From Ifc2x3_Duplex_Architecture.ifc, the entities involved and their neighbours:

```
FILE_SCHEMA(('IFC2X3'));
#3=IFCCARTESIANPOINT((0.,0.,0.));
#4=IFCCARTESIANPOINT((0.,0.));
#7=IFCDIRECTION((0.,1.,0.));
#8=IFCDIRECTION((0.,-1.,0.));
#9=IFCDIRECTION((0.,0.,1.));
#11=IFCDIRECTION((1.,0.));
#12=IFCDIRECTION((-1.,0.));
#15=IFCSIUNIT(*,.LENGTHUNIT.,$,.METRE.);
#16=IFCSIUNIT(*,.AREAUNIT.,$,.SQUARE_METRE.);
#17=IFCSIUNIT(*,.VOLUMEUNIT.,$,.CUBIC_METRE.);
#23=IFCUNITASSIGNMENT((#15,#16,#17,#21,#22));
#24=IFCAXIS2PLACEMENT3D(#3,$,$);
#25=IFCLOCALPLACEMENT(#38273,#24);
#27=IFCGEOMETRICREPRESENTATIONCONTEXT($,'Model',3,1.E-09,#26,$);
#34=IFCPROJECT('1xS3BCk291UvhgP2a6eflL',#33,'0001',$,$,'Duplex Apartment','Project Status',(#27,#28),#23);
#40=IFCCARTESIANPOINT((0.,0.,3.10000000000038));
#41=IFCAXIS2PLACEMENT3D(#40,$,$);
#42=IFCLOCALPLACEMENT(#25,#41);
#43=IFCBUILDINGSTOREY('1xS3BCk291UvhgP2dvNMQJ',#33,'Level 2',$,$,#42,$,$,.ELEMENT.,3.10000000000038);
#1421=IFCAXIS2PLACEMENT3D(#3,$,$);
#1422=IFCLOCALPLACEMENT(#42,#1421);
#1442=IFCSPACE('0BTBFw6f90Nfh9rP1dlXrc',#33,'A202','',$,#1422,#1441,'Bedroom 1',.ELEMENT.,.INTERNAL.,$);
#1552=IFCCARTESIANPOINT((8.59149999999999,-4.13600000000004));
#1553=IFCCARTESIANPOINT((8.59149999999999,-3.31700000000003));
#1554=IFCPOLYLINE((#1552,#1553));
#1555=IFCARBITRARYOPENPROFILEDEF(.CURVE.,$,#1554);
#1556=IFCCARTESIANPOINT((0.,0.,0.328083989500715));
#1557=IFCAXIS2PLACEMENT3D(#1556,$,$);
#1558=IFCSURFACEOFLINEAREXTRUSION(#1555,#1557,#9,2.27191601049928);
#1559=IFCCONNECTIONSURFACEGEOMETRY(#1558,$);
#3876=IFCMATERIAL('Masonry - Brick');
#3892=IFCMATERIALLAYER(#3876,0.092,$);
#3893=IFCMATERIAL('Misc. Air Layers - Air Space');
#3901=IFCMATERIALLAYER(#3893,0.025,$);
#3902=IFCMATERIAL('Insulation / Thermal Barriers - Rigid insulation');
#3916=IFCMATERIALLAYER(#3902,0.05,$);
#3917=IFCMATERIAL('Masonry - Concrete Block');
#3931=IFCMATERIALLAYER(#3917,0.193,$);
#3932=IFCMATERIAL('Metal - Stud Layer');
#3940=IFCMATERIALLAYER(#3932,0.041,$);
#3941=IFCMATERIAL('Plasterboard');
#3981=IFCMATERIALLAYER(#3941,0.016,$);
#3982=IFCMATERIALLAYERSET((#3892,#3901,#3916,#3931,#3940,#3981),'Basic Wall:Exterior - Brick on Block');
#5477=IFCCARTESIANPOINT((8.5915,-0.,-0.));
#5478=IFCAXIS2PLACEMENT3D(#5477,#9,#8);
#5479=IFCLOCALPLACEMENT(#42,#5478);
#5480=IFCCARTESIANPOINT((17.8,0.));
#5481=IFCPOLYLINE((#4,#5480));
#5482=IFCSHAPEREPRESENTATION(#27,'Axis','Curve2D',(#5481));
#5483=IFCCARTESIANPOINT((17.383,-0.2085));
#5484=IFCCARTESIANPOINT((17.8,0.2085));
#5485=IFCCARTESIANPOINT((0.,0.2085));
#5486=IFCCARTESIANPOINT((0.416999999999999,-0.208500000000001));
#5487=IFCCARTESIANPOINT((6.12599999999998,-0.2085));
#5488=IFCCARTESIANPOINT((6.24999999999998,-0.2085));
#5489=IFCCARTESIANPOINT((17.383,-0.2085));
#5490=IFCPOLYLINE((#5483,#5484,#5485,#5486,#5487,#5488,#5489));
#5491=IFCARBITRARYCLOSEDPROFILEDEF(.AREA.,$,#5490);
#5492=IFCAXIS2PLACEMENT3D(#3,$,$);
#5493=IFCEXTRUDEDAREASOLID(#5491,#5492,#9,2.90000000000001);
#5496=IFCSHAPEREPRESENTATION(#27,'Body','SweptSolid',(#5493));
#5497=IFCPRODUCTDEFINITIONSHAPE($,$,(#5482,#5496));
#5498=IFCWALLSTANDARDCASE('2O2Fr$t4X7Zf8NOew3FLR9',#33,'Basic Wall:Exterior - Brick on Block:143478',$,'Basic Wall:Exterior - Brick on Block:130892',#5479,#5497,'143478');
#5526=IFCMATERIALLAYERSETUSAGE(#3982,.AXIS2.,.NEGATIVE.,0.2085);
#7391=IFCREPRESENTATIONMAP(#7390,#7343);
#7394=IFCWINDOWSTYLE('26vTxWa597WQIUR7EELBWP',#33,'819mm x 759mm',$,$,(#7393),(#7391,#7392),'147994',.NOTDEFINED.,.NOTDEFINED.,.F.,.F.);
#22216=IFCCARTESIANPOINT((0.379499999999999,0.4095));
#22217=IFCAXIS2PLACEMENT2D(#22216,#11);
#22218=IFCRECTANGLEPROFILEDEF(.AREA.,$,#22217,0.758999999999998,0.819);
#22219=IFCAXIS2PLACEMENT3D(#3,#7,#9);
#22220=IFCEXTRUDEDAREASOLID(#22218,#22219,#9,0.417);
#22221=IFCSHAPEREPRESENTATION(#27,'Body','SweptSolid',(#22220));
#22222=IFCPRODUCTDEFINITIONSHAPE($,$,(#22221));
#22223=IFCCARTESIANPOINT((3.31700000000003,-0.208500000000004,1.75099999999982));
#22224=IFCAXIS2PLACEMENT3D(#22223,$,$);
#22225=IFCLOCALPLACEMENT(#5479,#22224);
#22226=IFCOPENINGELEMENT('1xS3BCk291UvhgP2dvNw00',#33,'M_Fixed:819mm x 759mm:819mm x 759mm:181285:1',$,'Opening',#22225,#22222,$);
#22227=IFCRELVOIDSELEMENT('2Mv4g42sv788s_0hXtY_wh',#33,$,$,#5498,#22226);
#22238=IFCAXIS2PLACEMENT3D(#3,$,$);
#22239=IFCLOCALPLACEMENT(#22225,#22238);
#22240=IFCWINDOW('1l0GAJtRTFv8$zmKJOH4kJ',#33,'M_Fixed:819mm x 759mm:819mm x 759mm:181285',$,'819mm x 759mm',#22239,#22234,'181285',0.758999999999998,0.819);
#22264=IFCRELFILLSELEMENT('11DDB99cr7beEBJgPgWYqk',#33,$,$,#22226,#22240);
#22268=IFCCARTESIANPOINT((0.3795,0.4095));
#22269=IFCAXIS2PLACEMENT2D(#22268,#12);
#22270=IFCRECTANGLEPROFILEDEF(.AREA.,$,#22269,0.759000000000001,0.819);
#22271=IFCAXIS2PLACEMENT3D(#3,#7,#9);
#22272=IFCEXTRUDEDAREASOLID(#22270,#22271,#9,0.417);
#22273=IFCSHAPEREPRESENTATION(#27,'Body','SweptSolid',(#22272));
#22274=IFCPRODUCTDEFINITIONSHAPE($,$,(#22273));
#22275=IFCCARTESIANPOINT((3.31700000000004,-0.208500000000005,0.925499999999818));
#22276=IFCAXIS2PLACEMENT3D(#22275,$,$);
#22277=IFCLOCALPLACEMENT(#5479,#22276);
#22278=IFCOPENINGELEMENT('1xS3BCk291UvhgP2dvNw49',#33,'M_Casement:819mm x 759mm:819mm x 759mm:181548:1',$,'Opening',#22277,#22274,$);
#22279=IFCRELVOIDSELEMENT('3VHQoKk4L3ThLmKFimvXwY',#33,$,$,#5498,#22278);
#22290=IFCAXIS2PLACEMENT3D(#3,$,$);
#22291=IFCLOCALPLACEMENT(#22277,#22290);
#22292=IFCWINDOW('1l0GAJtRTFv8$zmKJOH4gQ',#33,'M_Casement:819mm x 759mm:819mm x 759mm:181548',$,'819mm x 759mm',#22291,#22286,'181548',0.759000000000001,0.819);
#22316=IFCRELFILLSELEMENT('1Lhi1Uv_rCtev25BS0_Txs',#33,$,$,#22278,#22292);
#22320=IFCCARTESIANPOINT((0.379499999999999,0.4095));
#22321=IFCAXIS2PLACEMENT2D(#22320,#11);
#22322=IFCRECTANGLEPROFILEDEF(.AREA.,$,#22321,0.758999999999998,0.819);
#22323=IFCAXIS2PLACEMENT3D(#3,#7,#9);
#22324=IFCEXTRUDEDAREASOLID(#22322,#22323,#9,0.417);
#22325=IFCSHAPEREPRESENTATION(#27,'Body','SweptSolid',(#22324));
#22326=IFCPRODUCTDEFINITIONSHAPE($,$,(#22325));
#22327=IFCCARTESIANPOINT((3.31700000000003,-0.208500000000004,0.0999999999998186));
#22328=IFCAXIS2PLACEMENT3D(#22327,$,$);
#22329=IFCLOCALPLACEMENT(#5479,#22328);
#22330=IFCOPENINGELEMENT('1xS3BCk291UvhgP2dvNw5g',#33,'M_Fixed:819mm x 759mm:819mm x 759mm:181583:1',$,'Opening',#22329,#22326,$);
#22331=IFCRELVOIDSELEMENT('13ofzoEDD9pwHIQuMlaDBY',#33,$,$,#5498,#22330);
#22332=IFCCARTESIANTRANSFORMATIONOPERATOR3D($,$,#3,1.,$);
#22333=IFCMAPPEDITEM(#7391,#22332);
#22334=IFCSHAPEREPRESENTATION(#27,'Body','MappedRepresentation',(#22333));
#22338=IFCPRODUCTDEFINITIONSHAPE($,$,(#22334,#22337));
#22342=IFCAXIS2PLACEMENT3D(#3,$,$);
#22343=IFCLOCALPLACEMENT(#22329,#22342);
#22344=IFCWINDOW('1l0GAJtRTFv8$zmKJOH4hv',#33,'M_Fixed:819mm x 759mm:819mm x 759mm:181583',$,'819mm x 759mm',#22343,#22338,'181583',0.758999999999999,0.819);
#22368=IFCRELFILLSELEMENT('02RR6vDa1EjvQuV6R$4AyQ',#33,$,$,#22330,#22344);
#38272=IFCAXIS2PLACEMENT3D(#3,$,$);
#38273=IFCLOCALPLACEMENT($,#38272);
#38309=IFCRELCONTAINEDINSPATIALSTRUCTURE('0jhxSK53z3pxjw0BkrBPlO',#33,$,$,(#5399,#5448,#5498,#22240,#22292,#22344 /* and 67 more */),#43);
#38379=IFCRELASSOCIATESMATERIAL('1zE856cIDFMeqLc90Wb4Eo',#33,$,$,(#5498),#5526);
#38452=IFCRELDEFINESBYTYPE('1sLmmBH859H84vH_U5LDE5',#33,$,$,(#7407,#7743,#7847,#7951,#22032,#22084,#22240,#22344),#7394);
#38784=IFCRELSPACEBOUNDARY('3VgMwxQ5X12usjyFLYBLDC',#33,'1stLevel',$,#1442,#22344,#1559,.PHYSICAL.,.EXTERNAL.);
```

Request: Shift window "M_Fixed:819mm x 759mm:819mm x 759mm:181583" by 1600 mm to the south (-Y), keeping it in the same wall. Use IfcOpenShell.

```python
import numpy as np
import ifcopenshell
import ifcopenshell.api.geometry
import ifcopenshell.util.placement
import ifcopenshell.util.unit

model = ifcopenshell.open("Ifc2x3_Duplex_Architecture.ifc")
unit_scale = ifcopenshell.util.unit.calculate_unit_scale(model)

window = model.by_guid("1l0GAJtRTFv8$zmKJOH4hv")
opening = window.FillsVoids[0].RelatingOpeningElement
wall = opening.VoidsElements[0].RelatingBuildingElement

wall_matrix = ifcopenshell.util.placement.get_local_placement(wall.ObjectPlacement)
shift = wall_matrix[:3, 0] * 1.6 / unit_scale
before = ifcopenshell.util.placement.get_local_placement(window.ObjectPlacement)[:3, 3].copy()

# The window is placed relative to its opening, so it follows when the opening moves.
matrix = ifcopenshell.util.placement.get_local_placement(opening.ObjectPlacement)
matrix[:3, 3] += shift
ifcopenshell.api.geometry.edit_object_placement(
    model, product=opening, matrix=matrix, is_si=False, should_transform_children=True
)

# Space boundary surfaces are stored in each space's coordinates; move them too.
for rel in window.ProvidesBoundaries:
    if not rel.ConnectionGeometry:
        continue
    surface = rel.ConnectionGeometry.SurfaceOnRelatingElement
    space_matrix = ifcopenshell.util.placement.get_local_placement(rel.RelatingSpace.ObjectPlacement)
    point = np.array(surface.Position.Location.Coordinates) + space_matrix[:3, :3].T @ shift
    surface.Position = model.createIfcAxis2Placement3D(
        model.createIfcCartesianPoint(point.tolist()), surface.Position.Axis, surface.Position.RefDirection
    )

after = ifcopenshell.util.placement.get_local_placement(window.ObjectPlacement)[:3, 3]
print("window moved by", (after - before).round(3) + 0.0)

model.write("Ifc2x3_Duplex_Architecture_updated.ifc")
```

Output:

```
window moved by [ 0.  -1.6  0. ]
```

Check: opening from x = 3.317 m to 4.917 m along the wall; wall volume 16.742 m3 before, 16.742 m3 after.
